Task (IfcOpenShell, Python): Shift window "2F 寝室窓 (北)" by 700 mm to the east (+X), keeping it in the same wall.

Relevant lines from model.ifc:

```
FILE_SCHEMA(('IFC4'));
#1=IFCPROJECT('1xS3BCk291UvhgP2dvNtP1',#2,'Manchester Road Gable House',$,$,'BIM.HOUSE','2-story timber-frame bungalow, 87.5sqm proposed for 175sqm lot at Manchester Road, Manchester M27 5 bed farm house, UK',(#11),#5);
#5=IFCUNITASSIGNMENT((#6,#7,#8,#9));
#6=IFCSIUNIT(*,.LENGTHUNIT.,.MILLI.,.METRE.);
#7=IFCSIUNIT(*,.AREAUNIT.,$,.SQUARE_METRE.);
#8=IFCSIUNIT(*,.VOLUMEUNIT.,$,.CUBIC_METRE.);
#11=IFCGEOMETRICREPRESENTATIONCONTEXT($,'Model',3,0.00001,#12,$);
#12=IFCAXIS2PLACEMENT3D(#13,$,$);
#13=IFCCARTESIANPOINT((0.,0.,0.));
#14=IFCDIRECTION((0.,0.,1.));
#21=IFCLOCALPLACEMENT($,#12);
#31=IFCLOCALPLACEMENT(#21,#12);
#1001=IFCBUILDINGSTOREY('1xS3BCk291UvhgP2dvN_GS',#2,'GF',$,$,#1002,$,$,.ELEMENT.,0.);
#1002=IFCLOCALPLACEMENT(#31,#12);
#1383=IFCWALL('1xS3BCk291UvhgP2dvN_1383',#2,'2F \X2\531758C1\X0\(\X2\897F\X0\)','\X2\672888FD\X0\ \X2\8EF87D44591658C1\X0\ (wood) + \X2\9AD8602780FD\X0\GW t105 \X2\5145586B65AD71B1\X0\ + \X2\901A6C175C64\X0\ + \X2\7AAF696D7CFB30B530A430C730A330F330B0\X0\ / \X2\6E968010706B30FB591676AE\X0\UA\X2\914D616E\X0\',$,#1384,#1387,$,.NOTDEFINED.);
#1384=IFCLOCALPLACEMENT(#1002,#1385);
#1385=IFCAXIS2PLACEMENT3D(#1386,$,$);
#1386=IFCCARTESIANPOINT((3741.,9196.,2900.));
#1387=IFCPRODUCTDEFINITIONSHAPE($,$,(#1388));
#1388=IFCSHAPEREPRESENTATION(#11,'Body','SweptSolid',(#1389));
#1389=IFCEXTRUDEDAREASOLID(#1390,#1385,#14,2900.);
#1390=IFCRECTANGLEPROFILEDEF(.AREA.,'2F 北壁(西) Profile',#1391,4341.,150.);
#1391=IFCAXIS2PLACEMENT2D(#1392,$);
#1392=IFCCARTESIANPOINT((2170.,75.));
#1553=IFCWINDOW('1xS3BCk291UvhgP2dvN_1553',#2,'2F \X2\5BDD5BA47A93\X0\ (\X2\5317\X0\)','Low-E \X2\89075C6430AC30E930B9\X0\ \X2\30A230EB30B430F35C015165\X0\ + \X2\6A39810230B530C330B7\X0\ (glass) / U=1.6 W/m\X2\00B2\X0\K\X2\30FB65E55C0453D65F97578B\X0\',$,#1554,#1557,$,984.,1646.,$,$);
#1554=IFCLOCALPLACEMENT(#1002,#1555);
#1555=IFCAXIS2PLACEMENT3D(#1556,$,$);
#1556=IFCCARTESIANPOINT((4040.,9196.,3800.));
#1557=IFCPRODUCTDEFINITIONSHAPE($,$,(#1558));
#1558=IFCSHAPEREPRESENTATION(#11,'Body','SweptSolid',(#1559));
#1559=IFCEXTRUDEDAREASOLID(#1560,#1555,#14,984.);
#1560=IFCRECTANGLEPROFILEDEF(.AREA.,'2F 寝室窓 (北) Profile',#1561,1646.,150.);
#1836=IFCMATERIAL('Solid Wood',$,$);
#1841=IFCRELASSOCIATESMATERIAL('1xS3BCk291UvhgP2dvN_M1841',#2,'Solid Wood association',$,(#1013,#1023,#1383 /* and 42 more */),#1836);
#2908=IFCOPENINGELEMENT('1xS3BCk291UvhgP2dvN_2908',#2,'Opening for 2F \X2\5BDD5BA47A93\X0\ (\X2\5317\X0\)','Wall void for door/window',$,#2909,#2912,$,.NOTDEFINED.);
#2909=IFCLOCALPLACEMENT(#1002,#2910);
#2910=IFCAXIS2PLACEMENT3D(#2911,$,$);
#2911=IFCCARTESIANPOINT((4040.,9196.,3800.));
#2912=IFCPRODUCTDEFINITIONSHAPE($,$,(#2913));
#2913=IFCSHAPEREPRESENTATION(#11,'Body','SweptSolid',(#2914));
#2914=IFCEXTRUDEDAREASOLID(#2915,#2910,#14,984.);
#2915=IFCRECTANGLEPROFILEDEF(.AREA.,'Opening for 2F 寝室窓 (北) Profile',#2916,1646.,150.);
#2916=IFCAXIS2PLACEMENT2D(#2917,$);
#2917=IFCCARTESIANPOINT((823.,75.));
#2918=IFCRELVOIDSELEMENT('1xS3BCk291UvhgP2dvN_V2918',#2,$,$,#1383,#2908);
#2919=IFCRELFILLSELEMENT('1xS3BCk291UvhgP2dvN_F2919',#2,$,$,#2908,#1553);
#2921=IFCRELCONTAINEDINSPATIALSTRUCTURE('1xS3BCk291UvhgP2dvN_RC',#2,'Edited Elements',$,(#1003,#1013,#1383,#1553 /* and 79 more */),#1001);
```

```python
import ifcopenshell
import ifcopenshell.api.geometry
import ifcopenshell.util.placement

model = ifcopenshell.open("model.ifc")

window = model.by_id(1553)
opening = window.FillsVoids[0].RelatingOpeningElement
wall = opening.VoidsElements[0].RelatingBuildingElement

wall_matrix = ifcopenshell.util.placement.get_local_placement(wall.ObjectPlacement)
shift = wall_matrix[:3, 0] * 700.0
before = ifcopenshell.util.placement.get_local_placement(window.ObjectPlacement)[:3, 3].copy()

# The window is not placed relative to its opening, so move both.
for product in (opening, window):
    matrix = ifcopenshell.util.placement.get_local_placement(product.ObjectPlacement)
    matrix[:3, 3] += shift
    ifcopenshell.api.geometry.edit_object_placement(model, product=product, matrix=matrix, is_si=False)

after = ifcopenshell.util.placement.get_local_placement(window.ObjectPlacement)[:3, 3]
print("window moved by", (after - before).round(3) + 0.0)

model.write("model_rev.ifc")
```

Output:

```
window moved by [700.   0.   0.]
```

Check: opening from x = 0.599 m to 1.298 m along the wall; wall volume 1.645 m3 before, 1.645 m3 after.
